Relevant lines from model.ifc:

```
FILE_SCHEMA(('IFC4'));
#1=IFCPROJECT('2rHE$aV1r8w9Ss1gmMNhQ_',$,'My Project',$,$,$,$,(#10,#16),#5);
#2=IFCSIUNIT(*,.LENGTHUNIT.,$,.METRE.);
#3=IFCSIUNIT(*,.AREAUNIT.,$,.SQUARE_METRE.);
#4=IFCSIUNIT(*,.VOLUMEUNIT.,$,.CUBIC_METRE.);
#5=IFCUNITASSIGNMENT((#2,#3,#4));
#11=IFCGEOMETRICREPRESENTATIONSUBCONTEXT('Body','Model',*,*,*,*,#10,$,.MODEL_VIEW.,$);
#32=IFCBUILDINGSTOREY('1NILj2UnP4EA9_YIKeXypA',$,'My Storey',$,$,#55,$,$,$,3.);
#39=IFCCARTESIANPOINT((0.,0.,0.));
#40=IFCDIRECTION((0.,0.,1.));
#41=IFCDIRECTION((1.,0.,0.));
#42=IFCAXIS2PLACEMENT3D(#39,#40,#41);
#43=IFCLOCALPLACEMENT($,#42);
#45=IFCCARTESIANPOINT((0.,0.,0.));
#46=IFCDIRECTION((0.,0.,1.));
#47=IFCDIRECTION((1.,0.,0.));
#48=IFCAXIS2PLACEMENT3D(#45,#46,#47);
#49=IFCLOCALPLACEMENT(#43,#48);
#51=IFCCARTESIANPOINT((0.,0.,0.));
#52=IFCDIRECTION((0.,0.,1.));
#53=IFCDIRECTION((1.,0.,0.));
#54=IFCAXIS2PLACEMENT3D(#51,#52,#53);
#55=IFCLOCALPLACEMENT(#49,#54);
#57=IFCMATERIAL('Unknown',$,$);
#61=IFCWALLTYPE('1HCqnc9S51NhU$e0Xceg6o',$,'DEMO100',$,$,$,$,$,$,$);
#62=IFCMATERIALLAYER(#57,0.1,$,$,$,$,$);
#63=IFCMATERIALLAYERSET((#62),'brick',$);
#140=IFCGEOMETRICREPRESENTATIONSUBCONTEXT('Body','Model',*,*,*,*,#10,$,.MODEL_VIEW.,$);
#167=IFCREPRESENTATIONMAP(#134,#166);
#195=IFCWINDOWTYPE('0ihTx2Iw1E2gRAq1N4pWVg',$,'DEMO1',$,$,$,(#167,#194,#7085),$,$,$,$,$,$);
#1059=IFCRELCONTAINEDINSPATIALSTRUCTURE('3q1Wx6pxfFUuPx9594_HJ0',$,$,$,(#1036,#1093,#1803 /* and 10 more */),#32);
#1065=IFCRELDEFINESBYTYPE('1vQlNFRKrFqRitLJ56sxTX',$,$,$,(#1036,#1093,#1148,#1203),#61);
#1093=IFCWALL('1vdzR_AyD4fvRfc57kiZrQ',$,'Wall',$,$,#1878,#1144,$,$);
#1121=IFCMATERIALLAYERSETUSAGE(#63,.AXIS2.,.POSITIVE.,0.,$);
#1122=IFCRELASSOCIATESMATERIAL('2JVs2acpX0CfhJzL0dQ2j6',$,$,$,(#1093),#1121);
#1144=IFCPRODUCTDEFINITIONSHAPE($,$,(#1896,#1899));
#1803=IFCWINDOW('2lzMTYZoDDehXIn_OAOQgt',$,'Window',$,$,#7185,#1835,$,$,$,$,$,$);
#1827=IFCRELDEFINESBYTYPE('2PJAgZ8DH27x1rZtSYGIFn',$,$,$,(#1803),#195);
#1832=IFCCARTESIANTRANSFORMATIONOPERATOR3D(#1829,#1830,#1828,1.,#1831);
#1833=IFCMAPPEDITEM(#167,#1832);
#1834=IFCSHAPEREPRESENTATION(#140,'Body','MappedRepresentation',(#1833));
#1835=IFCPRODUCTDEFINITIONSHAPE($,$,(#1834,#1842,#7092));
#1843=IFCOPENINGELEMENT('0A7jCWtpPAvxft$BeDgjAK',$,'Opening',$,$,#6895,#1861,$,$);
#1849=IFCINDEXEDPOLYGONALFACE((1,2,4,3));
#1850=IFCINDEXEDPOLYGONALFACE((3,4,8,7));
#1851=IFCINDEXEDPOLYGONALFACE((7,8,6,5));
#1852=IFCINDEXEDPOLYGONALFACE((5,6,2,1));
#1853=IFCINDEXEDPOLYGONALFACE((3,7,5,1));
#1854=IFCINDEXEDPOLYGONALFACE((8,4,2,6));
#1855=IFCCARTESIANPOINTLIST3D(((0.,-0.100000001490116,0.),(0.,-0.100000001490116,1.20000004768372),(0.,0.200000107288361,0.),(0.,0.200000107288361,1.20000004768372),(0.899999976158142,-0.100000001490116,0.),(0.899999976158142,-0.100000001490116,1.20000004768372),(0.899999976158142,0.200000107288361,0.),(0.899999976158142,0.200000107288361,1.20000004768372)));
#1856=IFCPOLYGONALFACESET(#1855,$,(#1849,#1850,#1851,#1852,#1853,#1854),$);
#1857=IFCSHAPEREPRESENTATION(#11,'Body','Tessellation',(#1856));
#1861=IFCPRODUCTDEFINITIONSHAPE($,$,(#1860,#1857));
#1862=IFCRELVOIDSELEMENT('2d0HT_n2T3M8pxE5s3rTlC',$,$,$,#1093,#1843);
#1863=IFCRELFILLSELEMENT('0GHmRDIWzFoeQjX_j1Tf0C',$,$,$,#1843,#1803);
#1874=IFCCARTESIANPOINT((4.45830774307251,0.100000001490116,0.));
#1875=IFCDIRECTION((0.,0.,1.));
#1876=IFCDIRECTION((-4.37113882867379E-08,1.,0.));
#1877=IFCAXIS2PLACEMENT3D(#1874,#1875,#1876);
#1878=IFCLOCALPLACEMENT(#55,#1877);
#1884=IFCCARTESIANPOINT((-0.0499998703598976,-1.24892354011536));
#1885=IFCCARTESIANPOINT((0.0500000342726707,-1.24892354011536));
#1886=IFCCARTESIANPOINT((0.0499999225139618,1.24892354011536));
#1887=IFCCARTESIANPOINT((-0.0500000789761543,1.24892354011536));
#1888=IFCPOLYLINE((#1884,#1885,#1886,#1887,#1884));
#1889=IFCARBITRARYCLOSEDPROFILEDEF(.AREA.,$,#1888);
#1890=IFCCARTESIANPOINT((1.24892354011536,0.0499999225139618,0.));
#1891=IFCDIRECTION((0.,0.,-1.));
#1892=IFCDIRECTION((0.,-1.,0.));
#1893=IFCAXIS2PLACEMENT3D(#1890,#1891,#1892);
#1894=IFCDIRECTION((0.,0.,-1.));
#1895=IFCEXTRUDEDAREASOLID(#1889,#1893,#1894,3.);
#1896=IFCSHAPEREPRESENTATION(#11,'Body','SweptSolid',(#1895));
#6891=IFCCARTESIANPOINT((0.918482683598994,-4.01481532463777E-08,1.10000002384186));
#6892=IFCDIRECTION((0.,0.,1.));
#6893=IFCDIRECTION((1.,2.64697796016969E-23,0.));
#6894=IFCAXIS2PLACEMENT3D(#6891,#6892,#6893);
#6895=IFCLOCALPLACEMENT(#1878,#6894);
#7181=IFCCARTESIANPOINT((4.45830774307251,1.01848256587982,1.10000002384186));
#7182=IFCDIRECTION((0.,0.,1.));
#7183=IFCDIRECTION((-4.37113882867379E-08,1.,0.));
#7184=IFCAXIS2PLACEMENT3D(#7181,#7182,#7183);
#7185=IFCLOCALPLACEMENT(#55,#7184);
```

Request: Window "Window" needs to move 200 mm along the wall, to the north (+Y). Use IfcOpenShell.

```python
import ifcopenshell
import ifcopenshell.api.geometry
import ifcopenshell.util.placement
import ifcopenshell.util.unit

model = ifcopenshell.open("model.ifc")
unit_scale = ifcopenshell.util.unit.calculate_unit_scale(model)

window = model.by_guid("2lzMTYZoDDehXIn_OAOQgt")
opening = window.FillsVoids[0].RelatingOpeningElement
wall = opening.VoidsElements[0].RelatingBuildingElement

wall_matrix = ifcopenshell.util.placement.get_local_placement(wall.ObjectPlacement)
shift = wall_matrix[:3, 0] * 0.2 / unit_scale
before = ifcopenshell.util.placement.get_local_placement(window.ObjectPlacement)[:3, 3].copy()

# The window is not placed relative to its opening, so move both.
for product in (opening, window):
    matrix = ifcopenshell.util.placement.get_local_placement(product.ObjectPlacement)
    matrix[:3, 3] += shift
    ifcopenshell.api.geometry.edit_object_placement(model, product=product, matrix=matrix, is_si=False)

after = ifcopenshell.util.placement.get_local_placement(window.ObjectPlacement)[:3, 3]
print("window moved by", (after - before).round(3) + 0.0)

model.write("model_v2.ifc")
```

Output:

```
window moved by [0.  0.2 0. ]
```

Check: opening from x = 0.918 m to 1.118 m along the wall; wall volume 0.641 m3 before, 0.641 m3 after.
